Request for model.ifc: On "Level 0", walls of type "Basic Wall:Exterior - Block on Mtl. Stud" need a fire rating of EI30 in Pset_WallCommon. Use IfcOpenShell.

First a look at what the model holds.

```python
import ifcopenshell
import ifcopenshell.util.element

model = ifcopenshell.open("model.ifc")
print(model.schema)
storey = next(s for s in model.by_type("IfcBuildingStorey") if s.Name == "Level 0")
walls = [e for e in ifcopenshell.util.element.get_decomposition(storey) if e.is_a("IfcWall")]
seen = {}
for e in walls:
    element_type = ifcopenshell.util.element.get_type(e)
    key = (element_type.Name if element_type != e and element_type else None, ifcopenshell.util.element.get_pset(e, "Pset_WallCommon", "FireRating"))
    seen[key] = seen.get(key, 0) + 1
for (name, value), count in sorted(seen.items(), key=str):
    print(count, "x", name, "|", value)
```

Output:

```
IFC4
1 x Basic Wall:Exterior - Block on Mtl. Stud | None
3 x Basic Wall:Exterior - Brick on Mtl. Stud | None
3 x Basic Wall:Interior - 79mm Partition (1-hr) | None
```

```python
import ifcopenshell
import ifcopenshell.api.pset
import ifcopenshell.util.element

model = ifcopenshell.open("model.ifc")

storey = next(s for s in model.by_type("IfcBuildingStorey") if s.Name == "Level 0")
walls = [e for e in ifcopenshell.util.element.get_decomposition(storey) if e.is_a("IfcWall")]

count = 0
for e in walls:
    element_type = ifcopenshell.util.element.get_type(e)
    if element_type in (None, e) or element_type.Name != "Basic Wall:Exterior - Block on Mtl. Stud":
        continue
    # add_pset returns the element's existing set when there is one.
    pset = ifcopenshell.api.pset.add_pset(model, product=e, name="Pset_WallCommon")
    ifcopenshell.api.pset.edit_pset(model, pset=pset, properties={"FireRating": "EI30"})
    count += 1

print(count, "walls updated")

model.write("model-out.ifc")
```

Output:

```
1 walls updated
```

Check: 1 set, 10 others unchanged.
